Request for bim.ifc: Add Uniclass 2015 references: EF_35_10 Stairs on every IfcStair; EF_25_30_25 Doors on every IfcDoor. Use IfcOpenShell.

First a look at what the model holds.

```python
import ifcopenshell

model = ifcopenshell.open("bim.ifc")
print(model.schema)
print("classifications:", [c.Name for c in model.by_type("IfcClassification")])
for ifc_class in ("IfcDoor", "IfcRoof", "IfcStair", "IfcWall", "IfcWindow"):
    print(ifc_class, len(model.by_type(ifc_class)))
```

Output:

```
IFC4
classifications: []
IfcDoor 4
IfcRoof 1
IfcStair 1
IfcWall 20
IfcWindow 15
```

```python
import ifcopenshell
import ifcopenshell.api.classification

model = ifcopenshell.open("bim.ifc")

system = ifcopenshell.api.classification.add_classification(model, classification="Uniclass 2015")

codes = {
    "IfcStair": ("EF_35_10", "Stairs"),
    "IfcDoor": ("EF_25_30_25", "Doors"),
}
for ifc_class, (code, name) in codes.items():
    products = model.by_type(ifc_class)
    ifcopenshell.api.classification.add_reference(
        model, products=products, classification=system, identification=code, name=name
    )
    print(code, len(products))

model.write("bim_edited.ifc")
```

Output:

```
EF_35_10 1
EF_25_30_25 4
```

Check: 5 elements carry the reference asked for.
